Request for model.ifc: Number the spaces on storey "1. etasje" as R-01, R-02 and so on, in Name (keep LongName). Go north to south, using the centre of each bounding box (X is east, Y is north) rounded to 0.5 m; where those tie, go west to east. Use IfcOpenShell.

First a look at what the model holds.

```python
import ifcopenshell
import ifcopenshell.util.element
import ifcopenshell.util.placement

model = ifcopenshell.open("model.ifc")
print(model.schema)
storey = next(s for s in model.by_type("IfcBuildingStorey") if s.Name == "1. etasje")
spaces = [e for e in ifcopenshell.util.element.get_decomposition(storey) if e.is_a("IfcSpace")]
for e in sorted(spaces, key=lambda e: e.id()):
    origin = ifcopenshell.util.placement.get_local_placement(e.ObjectPlacement)[:3, 3]
    print(e.id(), e.Name, e.LongName, origin.round(2) + 0.0, sep=" | ")
```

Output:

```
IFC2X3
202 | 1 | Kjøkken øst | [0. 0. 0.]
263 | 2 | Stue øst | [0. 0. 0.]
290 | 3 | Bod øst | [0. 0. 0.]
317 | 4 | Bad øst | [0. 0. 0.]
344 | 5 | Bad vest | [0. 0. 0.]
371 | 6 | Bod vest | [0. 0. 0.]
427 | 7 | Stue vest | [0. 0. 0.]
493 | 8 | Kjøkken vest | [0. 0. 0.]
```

```python
import ifcopenshell
import ifcopenshell.geom
import ifcopenshell.util.element
import ifcopenshell.util.shape

model = ifcopenshell.open("model.ifc")
settings = ifcopenshell.geom.settings()
settings.set("use-world-coords", True)


def centre(element):
    shape = ifcopenshell.geom.create_shape(settings, element)
    return ifcopenshell.util.shape.get_bbox_centroid(shape.geometry)


storey = next(s for s in model.by_type("IfcBuildingStorey") if s.Name == "1. etasje")
spaces = [e for e in ifcopenshell.util.element.get_decomposition(storey) if e.is_a("IfcSpace")]

# Insertion points can sit at a corner or the storey origin, so sort by the geometry (in metres).
centres = {e: centre(e) for e in spaces}
spaces.sort(key=lambda e: (-round(centres[e][1] / 0.5), centres[e][0]))

for i, e in enumerate(spaces, start=1):
    number = f"R-{i:02d}"
    e.Name = number
    print(e.id(), number)

model.write("model_rev.ifc")
```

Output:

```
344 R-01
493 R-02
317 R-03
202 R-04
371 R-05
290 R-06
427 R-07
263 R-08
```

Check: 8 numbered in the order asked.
